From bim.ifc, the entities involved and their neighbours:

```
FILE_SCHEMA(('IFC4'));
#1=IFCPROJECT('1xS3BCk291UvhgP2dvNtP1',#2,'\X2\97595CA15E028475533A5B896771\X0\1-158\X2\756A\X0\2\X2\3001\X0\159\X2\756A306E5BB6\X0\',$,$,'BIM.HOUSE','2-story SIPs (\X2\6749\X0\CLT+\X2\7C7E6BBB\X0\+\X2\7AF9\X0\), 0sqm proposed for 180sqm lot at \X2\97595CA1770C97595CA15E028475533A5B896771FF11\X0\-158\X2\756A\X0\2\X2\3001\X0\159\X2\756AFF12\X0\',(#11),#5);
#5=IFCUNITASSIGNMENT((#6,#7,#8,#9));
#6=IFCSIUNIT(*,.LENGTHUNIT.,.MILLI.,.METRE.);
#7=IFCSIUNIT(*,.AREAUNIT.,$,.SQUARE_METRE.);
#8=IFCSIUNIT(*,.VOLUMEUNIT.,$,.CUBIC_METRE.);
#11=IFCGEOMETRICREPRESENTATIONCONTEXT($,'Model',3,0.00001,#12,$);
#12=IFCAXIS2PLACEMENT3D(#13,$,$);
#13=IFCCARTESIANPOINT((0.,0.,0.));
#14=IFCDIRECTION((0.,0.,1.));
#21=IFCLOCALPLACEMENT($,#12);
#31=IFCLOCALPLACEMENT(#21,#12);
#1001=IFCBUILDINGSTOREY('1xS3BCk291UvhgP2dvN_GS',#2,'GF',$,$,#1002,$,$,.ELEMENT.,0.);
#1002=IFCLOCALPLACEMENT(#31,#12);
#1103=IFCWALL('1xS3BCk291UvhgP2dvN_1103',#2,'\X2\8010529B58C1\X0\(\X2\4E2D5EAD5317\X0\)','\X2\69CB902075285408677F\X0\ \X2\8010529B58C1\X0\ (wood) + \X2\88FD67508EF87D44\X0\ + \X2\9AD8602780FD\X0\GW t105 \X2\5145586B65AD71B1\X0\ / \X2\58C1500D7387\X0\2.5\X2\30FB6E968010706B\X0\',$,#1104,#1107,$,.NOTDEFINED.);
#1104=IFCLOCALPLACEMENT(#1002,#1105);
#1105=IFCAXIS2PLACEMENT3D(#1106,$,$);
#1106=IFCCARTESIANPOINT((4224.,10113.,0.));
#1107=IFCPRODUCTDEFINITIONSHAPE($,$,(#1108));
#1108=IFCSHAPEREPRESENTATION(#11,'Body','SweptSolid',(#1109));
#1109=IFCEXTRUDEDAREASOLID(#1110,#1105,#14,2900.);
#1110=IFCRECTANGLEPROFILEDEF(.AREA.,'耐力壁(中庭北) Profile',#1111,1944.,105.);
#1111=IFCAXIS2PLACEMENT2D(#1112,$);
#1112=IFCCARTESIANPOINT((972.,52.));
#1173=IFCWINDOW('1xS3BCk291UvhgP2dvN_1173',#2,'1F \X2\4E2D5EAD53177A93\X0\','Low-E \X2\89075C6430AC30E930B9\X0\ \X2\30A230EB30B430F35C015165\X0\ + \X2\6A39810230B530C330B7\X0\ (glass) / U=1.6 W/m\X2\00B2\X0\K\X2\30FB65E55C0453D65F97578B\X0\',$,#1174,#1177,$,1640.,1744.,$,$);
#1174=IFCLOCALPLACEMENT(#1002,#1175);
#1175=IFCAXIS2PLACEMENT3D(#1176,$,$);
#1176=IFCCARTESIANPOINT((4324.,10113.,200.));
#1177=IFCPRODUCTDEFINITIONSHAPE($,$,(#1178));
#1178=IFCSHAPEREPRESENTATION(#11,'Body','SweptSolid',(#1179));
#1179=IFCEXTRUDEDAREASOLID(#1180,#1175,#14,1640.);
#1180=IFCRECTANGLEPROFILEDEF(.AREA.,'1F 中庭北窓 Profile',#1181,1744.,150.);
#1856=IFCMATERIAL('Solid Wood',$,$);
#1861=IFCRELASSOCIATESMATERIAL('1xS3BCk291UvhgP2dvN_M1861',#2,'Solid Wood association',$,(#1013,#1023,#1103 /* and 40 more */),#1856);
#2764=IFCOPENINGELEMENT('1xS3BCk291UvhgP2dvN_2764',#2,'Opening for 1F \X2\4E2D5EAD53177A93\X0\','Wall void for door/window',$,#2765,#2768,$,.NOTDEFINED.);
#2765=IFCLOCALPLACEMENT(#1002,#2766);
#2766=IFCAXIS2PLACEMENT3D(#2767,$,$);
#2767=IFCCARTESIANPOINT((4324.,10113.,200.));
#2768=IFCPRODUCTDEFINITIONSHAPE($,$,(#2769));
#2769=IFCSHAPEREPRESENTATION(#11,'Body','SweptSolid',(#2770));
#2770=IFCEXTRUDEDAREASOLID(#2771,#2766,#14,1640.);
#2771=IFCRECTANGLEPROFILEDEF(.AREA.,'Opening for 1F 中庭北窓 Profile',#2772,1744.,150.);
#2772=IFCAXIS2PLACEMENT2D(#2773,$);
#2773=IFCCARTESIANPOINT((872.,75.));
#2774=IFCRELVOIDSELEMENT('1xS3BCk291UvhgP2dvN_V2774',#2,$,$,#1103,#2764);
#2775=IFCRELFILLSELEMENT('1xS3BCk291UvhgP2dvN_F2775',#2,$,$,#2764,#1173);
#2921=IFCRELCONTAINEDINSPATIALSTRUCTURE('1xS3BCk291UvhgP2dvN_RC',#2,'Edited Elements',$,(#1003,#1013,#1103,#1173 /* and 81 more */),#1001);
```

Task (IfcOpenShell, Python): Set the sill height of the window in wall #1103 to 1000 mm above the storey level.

```python
import numpy as np
import ifcopenshell
import ifcopenshell.api.geometry
import ifcopenshell.geom
import ifcopenshell.util.element
import ifcopenshell.util.placement
import ifcopenshell.util.shape
import ifcopenshell.util.unit

model = ifcopenshell.open("bim.ifc")
unit_scale = ifcopenshell.util.unit.calculate_unit_scale(model)

window = model.by_guid("1xS3BCk291UvhgP2dvN_1173")
opening = window.FillsVoids[0].RelatingOpeningElement
storey = ifcopenshell.util.element.get_container(window, ifc_class="IfcBuildingStorey")
level = ifcopenshell.util.placement.get_local_placement(storey.ObjectPlacement)[2, 3]

# The opening's origin need not be at the sill, so measure its lowest point.
shape = ifcopenshell.geom.create_shape(ifcopenshell.geom.settings(), opening)
bottom = ifcopenshell.util.shape.get_shape_bottom_elevation(shape, shape.geometry) / unit_scale
dz = level + 1 / unit_scale - bottom

shift = np.array([0.0, 0.0, dz])
# The window is not placed relative to its opening, so move both.
for product in (opening, window):
    matrix = ifcopenshell.util.placement.get_local_placement(product.ObjectPlacement)
    matrix[:3, 3] += shift
    ifcopenshell.api.geometry.edit_object_placement(model, product=product, matrix=matrix, is_si=False)

print(f"moved by {dz * unit_scale:+.3f} m")

model.write("bim-out.ifc")
```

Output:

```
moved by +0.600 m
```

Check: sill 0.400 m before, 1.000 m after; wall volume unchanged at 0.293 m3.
